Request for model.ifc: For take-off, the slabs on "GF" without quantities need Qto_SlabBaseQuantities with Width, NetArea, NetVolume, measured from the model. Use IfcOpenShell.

First a look at what the model holds.

```python
import ifcopenshell
import ifcopenshell.util.element
import ifcopenshell.util.unit

model = ifcopenshell.open("model.ifc")
print(model.schema)
for unit_type in ("LENGTHUNIT", "AREAUNIT", "VOLUMEUNIT"):
    print(unit_type, ifcopenshell.util.unit.calculate_unit_scale(model, unit_type))
storey = next(s for s in model.by_type("IfcBuildingStorey") if s.Name == "GF")
slabs = [e for e in ifcopenshell.util.element.get_decomposition(storey) if e.is_a("IfcSlab")]
for e in sorted(slabs, key=lambda e: e.id()):
    print(e.id(), e.is_a(), e.Name, list(ifcopenshell.util.element.get_psets(e, qtos_only=True)), sep=" | ")
```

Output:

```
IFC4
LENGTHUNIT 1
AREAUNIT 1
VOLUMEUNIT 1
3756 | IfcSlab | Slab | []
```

```python
import ifcopenshell
import ifcopenshell.api.pset
import ifcopenshell.geom
import ifcopenshell.util.element
import ifcopenshell.util.shape
import ifcopenshell.util.unit

model = ifcopenshell.open("model.ifc")
unit_scale = ifcopenshell.util.unit.calculate_unit_scale(model)
area_scale = ifcopenshell.util.unit.calculate_unit_scale(model, "AREAUNIT")
volume_scale = ifcopenshell.util.unit.calculate_unit_scale(model, "VOLUMEUNIT")
settings = ifcopenshell.geom.settings()

storey = next(s for s in model.by_type("IfcBuildingStorey") if s.Name == "GF")
slabs = [e for e in ifcopenshell.util.element.get_decomposition(storey) if e.is_a("IfcSlab")]

for e in sorted(slabs, key=lambda e: e.id()):
    if ifcopenshell.util.element.get_psets(e, qtos_only=True, should_inherit=False):
        continue
    # Geometry comes back in metres, in the element's own axes.
    shape = ifcopenshell.geom.create_shape(settings, e)
    values = {
        "Width": ifcopenshell.util.shape.get_z(shape.geometry) / unit_scale,
        "NetArea": ifcopenshell.util.shape.get_footprint_area(shape.geometry) / area_scale,
        "NetVolume": ifcopenshell.util.shape.get_volume(shape.geometry) / volume_scale,
    }
    qto = ifcopenshell.api.pset.add_qto(model, product=e, name="Qto_SlabBaseQuantities")
    ifcopenshell.api.pset.edit_qto(model, qto=qto, properties=values)
    print(e.id(), {k: round(v, 3) for k, v in values.items()})

model.write("model_updated.ifc")
```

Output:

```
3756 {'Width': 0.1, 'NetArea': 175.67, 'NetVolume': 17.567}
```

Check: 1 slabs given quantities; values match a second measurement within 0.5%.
